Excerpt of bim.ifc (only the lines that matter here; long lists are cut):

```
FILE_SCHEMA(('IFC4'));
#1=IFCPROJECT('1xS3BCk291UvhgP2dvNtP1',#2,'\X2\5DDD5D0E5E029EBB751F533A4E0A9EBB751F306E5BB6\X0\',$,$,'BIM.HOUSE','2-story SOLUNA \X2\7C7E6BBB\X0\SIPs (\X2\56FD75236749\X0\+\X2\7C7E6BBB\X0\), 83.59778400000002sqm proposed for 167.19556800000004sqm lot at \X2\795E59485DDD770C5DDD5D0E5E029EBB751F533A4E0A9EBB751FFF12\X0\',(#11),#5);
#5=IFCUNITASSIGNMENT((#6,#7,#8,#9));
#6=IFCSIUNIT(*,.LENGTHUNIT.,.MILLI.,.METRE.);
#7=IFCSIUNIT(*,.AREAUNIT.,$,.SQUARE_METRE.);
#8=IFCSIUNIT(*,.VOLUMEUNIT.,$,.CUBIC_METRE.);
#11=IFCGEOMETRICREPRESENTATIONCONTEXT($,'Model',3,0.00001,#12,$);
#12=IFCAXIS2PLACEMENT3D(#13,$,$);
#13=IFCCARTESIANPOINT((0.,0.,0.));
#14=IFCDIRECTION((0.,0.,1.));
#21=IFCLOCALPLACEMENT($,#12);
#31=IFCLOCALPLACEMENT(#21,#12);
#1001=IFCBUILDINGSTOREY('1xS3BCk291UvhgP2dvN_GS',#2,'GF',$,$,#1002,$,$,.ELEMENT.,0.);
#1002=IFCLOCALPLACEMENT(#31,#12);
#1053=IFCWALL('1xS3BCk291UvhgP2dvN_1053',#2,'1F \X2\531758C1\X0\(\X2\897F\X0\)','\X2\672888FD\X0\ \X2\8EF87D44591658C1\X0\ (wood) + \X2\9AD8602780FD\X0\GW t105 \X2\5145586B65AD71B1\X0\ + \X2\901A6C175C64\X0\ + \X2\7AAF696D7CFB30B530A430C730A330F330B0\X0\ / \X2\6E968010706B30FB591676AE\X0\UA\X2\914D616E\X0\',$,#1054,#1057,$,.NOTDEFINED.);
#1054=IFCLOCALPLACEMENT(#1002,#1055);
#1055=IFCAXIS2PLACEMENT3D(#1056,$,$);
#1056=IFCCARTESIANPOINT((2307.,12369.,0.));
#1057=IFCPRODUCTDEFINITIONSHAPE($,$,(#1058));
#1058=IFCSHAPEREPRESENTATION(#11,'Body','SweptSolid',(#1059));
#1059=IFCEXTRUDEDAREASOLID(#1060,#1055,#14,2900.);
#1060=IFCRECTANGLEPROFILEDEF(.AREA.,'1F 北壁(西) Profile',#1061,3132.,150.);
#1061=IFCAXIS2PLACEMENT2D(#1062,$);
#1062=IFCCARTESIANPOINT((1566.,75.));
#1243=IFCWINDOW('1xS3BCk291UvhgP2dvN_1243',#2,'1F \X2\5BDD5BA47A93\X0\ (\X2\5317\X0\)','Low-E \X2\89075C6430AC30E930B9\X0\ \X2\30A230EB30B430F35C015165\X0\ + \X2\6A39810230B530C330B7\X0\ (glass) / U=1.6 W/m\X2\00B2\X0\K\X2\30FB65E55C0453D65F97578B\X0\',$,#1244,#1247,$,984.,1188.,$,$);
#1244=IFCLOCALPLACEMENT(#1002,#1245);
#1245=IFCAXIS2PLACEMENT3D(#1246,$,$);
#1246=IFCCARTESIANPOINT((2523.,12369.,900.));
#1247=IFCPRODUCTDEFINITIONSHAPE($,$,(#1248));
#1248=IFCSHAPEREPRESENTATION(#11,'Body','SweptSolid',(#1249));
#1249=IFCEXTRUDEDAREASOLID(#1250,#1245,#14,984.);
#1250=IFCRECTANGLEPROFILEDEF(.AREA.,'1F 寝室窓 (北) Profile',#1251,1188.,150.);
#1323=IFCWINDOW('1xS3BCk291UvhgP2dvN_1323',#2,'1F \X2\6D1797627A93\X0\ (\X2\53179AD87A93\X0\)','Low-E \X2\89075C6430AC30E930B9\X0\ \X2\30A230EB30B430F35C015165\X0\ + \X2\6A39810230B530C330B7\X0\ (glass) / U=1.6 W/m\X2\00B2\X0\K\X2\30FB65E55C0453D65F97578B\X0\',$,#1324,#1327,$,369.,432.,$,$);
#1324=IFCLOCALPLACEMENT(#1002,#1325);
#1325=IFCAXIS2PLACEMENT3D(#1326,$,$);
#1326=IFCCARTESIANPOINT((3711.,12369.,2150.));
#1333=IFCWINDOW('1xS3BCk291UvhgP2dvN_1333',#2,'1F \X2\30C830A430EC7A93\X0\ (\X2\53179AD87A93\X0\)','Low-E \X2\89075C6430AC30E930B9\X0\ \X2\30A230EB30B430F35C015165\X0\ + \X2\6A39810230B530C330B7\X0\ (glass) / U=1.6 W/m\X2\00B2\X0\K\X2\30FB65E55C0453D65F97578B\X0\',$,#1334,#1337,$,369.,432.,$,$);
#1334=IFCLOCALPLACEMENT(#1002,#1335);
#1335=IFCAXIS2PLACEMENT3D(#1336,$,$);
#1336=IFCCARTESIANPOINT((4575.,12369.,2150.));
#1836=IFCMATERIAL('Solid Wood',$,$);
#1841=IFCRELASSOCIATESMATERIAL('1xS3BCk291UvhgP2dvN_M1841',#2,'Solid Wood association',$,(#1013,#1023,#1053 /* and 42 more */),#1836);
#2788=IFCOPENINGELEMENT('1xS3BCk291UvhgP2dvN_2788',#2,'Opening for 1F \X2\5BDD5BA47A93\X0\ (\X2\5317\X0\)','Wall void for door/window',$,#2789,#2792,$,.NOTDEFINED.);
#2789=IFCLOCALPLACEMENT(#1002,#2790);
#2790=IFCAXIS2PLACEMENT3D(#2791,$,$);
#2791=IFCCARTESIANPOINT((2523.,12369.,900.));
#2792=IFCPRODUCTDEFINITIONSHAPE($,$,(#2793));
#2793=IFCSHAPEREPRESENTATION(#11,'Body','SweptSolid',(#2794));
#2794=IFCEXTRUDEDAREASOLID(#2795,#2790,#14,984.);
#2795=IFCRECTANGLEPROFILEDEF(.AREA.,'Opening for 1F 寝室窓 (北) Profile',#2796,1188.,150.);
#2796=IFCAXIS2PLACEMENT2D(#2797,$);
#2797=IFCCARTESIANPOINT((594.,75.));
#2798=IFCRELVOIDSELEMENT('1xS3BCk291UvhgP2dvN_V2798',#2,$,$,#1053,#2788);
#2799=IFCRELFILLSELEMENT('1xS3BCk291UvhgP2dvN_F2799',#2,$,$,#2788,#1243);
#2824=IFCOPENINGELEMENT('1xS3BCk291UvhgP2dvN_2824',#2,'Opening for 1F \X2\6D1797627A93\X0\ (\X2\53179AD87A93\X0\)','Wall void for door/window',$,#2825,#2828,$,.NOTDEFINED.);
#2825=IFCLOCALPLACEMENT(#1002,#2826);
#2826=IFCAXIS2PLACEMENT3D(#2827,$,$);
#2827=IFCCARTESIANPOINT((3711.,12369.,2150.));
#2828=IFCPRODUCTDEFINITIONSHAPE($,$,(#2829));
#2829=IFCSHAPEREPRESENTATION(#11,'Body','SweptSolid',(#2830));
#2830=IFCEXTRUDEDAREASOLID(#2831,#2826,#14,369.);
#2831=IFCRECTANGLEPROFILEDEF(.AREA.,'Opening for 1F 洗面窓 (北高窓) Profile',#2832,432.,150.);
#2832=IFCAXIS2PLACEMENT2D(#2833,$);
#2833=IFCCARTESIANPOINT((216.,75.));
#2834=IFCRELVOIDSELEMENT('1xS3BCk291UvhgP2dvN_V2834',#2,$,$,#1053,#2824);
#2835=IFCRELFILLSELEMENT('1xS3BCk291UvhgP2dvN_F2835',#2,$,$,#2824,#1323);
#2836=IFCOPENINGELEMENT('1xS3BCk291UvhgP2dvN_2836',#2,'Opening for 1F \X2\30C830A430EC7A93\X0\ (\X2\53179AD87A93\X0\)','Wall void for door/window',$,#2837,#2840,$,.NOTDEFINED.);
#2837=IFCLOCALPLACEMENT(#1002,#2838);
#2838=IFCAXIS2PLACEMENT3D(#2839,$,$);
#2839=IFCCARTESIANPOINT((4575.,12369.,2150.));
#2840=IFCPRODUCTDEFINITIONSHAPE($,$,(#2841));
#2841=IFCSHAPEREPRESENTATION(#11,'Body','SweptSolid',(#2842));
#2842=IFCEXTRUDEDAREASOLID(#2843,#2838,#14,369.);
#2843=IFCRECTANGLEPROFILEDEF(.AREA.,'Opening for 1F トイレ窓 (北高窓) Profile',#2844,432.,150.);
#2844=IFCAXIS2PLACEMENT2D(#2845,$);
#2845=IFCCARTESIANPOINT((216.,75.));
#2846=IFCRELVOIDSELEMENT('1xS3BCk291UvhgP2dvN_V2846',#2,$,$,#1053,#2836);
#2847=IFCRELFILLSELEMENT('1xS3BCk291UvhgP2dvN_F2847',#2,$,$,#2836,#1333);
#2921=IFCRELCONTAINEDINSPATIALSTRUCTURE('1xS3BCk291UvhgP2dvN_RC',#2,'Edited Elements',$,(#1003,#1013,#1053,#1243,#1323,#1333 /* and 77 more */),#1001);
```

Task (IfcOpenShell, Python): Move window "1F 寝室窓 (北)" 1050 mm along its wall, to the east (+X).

```python
import ifcopenshell
import ifcopenshell.api.geometry
import ifcopenshell.util.placement
import ifcopenshell.util.unit

model = ifcopenshell.open("bim.ifc")
unit_scale = ifcopenshell.util.unit.calculate_unit_scale(model)

window = model.by_guid("1xS3BCk291UvhgP2dvN_1243")
opening = window.FillsVoids[0].RelatingOpeningElement
wall = opening.VoidsElements[0].RelatingBuildingElement

wall_matrix = ifcopenshell.util.placement.get_local_placement(wall.ObjectPlacement)
shift = wall_matrix[:3, 0] * 1.05 / unit_scale
before = ifcopenshell.util.placement.get_local_placement(window.ObjectPlacement)[:3, 3].copy()

# The window is not placed relative to its opening, so move both.
for product in (opening, window):
    matrix = ifcopenshell.util.placement.get_local_placement(product.ObjectPlacement)
    matrix[:3, 3] += shift
    ifcopenshell.api.geometry.edit_object_placement(model, product=product, matrix=matrix, is_si=False)

after = ifcopenshell.util.placement.get_local_placement(window.ObjectPlacement)[:3, 3]
print("window moved by", (after - before).round(3) + 0.0)

model.write("bim_rev.ifc")
```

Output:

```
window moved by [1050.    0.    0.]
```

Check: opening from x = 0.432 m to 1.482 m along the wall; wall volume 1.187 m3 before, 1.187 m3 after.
